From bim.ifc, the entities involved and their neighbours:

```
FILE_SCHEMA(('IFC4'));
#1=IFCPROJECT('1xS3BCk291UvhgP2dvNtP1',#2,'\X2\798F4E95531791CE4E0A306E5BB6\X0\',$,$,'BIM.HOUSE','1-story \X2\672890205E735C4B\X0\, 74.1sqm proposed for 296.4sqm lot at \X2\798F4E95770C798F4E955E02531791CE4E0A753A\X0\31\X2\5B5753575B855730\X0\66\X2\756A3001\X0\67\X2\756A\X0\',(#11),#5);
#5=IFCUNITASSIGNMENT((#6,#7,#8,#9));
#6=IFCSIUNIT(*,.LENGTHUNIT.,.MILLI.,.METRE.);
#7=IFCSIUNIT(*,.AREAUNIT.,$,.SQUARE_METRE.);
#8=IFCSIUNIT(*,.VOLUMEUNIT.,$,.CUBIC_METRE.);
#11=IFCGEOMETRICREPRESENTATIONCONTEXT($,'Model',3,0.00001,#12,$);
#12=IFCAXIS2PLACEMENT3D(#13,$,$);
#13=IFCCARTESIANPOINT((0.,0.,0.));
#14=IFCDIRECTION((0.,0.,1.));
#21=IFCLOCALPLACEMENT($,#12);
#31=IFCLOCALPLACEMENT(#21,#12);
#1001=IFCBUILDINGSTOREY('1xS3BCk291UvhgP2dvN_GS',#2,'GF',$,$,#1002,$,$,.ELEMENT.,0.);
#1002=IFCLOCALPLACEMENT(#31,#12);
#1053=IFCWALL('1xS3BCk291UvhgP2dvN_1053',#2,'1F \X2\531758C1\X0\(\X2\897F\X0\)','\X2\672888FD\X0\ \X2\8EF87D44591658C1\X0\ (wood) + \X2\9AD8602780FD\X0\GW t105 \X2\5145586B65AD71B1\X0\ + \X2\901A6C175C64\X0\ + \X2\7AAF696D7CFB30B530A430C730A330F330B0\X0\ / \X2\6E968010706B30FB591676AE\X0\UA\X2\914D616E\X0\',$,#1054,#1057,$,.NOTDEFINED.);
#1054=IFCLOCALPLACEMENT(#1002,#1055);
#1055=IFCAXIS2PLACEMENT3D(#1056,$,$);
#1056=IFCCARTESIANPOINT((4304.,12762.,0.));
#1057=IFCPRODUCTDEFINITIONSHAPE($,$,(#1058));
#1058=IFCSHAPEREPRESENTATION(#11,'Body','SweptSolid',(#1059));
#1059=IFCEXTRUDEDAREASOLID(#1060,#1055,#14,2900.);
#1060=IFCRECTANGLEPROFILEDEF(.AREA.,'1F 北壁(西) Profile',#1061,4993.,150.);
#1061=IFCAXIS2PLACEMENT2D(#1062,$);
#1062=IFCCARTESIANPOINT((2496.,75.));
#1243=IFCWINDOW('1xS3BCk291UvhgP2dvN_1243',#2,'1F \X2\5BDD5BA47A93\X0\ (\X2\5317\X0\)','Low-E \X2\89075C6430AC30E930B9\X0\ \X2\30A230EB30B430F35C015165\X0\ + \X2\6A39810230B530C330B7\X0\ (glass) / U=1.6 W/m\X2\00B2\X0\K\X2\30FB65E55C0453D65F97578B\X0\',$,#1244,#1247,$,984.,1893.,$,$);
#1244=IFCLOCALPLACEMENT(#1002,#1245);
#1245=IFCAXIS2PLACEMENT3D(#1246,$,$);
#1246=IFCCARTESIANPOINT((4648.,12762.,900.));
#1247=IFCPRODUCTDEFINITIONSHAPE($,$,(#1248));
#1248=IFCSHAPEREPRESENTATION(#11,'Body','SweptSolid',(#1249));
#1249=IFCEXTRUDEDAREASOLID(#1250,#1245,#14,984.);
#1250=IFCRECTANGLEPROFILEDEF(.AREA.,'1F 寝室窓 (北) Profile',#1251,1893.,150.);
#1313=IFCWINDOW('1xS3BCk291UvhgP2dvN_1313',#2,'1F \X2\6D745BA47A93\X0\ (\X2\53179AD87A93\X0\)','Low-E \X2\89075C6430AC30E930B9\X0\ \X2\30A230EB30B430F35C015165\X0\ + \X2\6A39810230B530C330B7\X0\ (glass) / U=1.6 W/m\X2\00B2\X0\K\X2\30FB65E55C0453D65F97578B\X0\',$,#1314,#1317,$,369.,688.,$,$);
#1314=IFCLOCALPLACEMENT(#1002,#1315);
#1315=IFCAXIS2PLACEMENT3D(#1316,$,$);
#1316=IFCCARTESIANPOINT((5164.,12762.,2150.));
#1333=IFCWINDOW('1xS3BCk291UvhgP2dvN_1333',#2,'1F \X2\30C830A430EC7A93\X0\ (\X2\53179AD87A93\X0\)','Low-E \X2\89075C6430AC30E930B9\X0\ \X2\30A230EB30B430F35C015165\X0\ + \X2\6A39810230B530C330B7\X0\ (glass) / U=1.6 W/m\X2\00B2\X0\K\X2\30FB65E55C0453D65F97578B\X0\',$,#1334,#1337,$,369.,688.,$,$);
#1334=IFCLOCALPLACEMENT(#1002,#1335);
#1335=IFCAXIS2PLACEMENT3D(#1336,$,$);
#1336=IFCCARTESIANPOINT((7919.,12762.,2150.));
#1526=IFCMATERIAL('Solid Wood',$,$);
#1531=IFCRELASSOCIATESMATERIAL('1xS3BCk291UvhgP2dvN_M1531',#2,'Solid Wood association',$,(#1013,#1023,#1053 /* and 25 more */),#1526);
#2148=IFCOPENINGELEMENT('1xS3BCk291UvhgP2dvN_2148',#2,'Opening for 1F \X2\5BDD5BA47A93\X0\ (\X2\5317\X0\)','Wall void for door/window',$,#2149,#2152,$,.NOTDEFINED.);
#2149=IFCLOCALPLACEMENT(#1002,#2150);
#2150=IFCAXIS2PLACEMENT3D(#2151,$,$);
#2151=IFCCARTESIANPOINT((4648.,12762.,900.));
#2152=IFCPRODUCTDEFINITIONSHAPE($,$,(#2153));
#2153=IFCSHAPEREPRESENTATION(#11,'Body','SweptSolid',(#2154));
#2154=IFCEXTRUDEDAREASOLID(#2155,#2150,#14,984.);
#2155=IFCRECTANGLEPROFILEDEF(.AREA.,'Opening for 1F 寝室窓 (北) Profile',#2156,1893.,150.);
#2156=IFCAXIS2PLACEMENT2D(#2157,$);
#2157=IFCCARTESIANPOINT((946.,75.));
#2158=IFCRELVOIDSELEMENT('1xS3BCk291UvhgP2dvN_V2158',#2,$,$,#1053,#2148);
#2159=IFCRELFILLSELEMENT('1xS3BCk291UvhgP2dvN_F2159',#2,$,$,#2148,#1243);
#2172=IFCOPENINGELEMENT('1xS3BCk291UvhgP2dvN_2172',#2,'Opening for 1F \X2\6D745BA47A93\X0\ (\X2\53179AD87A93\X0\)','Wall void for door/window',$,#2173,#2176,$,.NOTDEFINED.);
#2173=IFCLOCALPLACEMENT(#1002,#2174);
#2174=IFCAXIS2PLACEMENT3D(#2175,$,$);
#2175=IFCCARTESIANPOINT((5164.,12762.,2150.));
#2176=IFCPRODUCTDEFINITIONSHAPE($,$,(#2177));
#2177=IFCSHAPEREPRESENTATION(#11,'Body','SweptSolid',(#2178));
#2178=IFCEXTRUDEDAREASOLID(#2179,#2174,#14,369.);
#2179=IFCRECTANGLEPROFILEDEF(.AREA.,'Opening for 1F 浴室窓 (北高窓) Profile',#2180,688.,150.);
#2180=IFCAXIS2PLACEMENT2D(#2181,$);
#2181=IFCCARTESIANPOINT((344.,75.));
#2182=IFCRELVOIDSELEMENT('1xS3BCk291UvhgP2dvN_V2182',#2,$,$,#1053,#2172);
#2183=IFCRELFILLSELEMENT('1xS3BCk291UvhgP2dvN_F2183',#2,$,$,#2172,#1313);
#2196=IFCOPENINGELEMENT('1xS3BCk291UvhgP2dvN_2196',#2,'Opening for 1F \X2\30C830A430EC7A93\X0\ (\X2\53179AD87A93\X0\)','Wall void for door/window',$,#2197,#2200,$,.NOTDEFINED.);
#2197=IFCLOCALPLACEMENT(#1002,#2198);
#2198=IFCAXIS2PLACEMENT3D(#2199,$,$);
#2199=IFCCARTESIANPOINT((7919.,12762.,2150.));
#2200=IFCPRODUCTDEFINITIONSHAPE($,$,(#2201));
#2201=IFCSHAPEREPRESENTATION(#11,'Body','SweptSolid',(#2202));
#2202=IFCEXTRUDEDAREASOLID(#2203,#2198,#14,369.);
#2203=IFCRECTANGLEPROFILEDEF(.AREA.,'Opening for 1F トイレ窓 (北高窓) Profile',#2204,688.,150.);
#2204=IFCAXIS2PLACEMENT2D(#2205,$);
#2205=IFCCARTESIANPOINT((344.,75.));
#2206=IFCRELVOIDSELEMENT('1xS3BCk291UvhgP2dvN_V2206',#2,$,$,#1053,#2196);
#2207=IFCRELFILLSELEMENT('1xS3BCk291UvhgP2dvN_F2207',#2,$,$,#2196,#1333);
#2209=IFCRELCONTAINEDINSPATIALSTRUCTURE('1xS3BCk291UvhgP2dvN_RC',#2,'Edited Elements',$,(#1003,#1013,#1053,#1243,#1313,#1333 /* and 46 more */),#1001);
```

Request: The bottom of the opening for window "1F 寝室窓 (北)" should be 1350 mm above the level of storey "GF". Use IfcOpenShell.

```python
import numpy as np
import ifcopenshell
import ifcopenshell.api.geometry
import ifcopenshell.geom
import ifcopenshell.util.element
import ifcopenshell.util.placement
import ifcopenshell.util.shape
import ifcopenshell.util.unit

model = ifcopenshell.open("bim.ifc")
unit_scale = ifcopenshell.util.unit.calculate_unit_scale(model)

window = model.by_guid("1xS3BCk291UvhgP2dvN_1243")
opening = window.FillsVoids[0].RelatingOpeningElement
storey = ifcopenshell.util.element.get_container(window, ifc_class="IfcBuildingStorey")
level = ifcopenshell.util.placement.get_local_placement(storey.ObjectPlacement)[2, 3]

# The opening's origin need not be at the sill, so measure its lowest point.
shape = ifcopenshell.geom.create_shape(ifcopenshell.geom.settings(), opening)
bottom = ifcopenshell.util.shape.get_shape_bottom_elevation(shape, shape.geometry) / unit_scale
dz = level + 1.35 / unit_scale - bottom

shift = np.array([0.0, 0.0, dz])
# The window is not placed relative to its opening, so move both.
for product in (opening, window):
    matrix = ifcopenshell.util.placement.get_local_placement(product.ObjectPlacement)
    matrix[:3, 3] += shift
    ifcopenshell.api.geometry.edit_object_placement(model, product=product, matrix=matrix, is_si=False)

print(f"moved by {dz * unit_scale:+.3f} m")

model.write("bim-out.ifc")
```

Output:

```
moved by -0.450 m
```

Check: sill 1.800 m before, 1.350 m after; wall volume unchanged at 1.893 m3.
